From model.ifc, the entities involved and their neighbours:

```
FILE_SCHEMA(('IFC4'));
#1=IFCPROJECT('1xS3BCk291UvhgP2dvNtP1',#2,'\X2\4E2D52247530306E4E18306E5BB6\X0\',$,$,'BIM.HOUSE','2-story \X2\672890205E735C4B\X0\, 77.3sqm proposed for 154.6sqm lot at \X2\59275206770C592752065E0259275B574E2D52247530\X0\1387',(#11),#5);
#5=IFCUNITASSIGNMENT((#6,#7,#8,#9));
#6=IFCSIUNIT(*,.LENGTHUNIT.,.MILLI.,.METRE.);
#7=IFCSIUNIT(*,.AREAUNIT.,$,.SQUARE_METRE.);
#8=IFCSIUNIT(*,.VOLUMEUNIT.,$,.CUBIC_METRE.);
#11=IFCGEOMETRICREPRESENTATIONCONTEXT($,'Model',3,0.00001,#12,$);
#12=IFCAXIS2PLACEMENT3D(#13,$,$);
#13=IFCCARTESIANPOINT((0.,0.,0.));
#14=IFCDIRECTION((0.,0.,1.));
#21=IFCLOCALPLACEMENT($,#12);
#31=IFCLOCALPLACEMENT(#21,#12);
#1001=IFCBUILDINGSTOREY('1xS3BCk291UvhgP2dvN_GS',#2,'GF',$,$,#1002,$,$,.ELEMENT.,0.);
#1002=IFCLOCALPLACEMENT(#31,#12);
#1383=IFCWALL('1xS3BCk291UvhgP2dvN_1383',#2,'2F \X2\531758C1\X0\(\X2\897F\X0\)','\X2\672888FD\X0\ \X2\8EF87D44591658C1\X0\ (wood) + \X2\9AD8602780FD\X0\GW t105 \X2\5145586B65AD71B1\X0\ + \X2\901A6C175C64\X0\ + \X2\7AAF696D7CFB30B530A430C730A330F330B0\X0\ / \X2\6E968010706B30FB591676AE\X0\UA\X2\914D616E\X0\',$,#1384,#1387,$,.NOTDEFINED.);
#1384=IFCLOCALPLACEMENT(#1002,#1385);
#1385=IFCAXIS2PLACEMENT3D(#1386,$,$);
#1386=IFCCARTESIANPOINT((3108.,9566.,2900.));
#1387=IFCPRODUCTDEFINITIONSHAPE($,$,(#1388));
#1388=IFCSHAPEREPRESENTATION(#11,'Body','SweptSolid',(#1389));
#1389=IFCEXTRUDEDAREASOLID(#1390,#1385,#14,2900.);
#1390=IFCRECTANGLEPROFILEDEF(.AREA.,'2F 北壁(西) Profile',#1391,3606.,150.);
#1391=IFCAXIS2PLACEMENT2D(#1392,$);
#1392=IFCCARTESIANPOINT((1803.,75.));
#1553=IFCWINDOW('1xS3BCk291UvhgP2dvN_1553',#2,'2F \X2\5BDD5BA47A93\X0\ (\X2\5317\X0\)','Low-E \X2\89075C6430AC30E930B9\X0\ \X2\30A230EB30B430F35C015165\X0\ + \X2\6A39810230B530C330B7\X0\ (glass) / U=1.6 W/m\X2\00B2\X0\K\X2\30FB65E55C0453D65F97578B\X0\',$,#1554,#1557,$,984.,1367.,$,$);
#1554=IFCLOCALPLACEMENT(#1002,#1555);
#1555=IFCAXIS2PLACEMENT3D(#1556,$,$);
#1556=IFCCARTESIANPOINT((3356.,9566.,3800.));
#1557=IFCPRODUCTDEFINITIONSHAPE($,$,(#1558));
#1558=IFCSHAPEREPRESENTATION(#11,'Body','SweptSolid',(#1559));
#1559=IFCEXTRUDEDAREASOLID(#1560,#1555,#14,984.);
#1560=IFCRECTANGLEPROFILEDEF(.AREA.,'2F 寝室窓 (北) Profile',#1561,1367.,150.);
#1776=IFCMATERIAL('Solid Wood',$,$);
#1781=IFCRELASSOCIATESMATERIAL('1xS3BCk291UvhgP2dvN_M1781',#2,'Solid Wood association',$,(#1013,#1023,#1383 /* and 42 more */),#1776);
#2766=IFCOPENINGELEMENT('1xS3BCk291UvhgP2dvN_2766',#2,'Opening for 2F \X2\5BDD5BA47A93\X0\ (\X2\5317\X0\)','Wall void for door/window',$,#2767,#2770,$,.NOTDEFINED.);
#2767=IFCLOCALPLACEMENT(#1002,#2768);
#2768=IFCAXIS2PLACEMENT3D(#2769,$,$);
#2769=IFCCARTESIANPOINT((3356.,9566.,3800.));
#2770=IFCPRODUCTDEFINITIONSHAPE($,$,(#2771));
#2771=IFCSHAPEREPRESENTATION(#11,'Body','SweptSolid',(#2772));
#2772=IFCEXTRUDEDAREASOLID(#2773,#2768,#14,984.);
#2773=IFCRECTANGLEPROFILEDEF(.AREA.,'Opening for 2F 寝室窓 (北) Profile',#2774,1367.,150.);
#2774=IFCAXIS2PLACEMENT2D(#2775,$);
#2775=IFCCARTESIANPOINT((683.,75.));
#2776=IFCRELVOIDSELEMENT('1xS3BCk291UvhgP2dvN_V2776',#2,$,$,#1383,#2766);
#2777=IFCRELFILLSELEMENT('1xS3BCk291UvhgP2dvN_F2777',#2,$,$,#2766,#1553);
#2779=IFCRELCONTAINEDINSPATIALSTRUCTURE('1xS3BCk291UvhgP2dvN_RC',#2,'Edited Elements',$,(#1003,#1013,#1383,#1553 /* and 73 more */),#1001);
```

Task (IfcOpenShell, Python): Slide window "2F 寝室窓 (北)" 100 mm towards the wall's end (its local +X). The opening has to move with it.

```python
import ifcopenshell
import ifcopenshell.api.geometry
import ifcopenshell.util.placement
import ifcopenshell.util.unit

model = ifcopenshell.open("model.ifc")
unit_scale = ifcopenshell.util.unit.calculate_unit_scale(model)

window = model.by_guid("1xS3BCk291UvhgP2dvN_1553")
opening = window.FillsVoids[0].RelatingOpeningElement
wall = opening.VoidsElements[0].RelatingBuildingElement

wall_matrix = ifcopenshell.util.placement.get_local_placement(wall.ObjectPlacement)
shift = wall_matrix[:3, 0] * 0.1 / unit_scale
before = ifcopenshell.util.placement.get_local_placement(window.ObjectPlacement)[:3, 3].copy()

# The window is not placed relative to its opening, so move both.
for product in (opening, window):
    matrix = ifcopenshell.util.placement.get_local_placement(product.ObjectPlacement)
    matrix[:3, 3] += shift
    ifcopenshell.api.geometry.edit_object_placement(model, product=product, matrix=matrix, is_si=False)

after = ifcopenshell.util.placement.get_local_placement(window.ObjectPlacement)[:3, 3]
print("window moved by", (after - before).round(3) + 0.0)

model.write("model-out.ifc")
```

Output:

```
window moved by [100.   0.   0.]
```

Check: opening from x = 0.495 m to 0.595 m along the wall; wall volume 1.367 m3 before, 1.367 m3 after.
